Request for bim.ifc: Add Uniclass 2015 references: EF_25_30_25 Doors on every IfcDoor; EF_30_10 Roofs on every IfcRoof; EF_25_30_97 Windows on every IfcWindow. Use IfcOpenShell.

First a look at what the model holds.

```python
import ifcopenshell

model = ifcopenshell.open("bim.ifc")
print(model.schema)
print("classifications:", [c.Name for c in model.by_type("IfcClassification")])
for ifc_class in ("IfcDoor", "IfcRoof", "IfcStair", "IfcWall", "IfcWindow"):
    print(ifc_class, len(model.by_type(ifc_class)))
```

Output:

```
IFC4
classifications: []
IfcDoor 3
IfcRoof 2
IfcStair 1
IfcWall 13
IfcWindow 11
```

```python
import ifcopenshell
import ifcopenshell.api.classification

model = ifcopenshell.open("bim.ifc")

system = ifcopenshell.api.classification.add_classification(model, classification="Uniclass 2015")

codes = {
    "IfcDoor": ("EF_25_30_25", "Doors"),
    "IfcRoof": ("EF_30_10", "Roofs"),
    "IfcWindow": ("EF_25_30_97", "Windows"),
}
for ifc_class, (code, name) in codes.items():
    products = model.by_type(ifc_class)
    ifcopenshell.api.classification.add_reference(
        model, products=products, classification=system, identification=code, name=name
    )
    print(code, len(products))

model.write("bim_rev.ifc")
```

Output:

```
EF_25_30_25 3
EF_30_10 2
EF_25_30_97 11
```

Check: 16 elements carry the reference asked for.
